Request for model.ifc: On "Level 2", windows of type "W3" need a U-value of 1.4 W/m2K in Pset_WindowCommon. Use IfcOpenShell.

First a look at what the model holds.

```python
import ifcopenshell
import ifcopenshell.util.element

model = ifcopenshell.open("model.ifc")
print(model.schema)
storey = next(s for s in model.by_type("IfcBuildingStorey") if s.Name == "Level 2")
windows = [e for e in ifcopenshell.util.element.get_decomposition(storey) if e.is_a("IfcWindow")]
seen = {}
for e in windows:
    element_type = ifcopenshell.util.element.get_type(e)
    key = (element_type.Name if element_type != e and element_type else None, ifcopenshell.util.element.get_pset(e, "Pset_WindowCommon", "ThermalTransmittance"))
    seen[key] = seen.get(key, 0) + 1
for (name, value), count in sorted(seen.items(), key=str):
    print(count, "x", name, "|", value)
```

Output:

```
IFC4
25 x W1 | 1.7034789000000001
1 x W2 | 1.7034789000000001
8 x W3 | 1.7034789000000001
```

```python
import ifcopenshell
import ifcopenshell.api.pset
import ifcopenshell.util.element

model = ifcopenshell.open("model.ifc")

storey = next(s for s in model.by_type("IfcBuildingStorey") if s.Name == "Level 2")
windows = [e for e in ifcopenshell.util.element.get_decomposition(storey) if e.is_a("IfcWindow")]

count = 0
for e in windows:
    element_type = ifcopenshell.util.element.get_type(e)
    if element_type in (None, e) or element_type.Name != "W3":
        continue
    # add_pset returns the element's existing set when there is one.
    pset = ifcopenshell.api.pset.add_pset(model, product=e, name="Pset_WindowCommon")
    ifcopenshell.api.pset.edit_pset(model, pset=pset, properties={"ThermalTransmittance": 1.4})
    count += 1

print(count, "windows updated")

model.write("model_updated.ifc")
```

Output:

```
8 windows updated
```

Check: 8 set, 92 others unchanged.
